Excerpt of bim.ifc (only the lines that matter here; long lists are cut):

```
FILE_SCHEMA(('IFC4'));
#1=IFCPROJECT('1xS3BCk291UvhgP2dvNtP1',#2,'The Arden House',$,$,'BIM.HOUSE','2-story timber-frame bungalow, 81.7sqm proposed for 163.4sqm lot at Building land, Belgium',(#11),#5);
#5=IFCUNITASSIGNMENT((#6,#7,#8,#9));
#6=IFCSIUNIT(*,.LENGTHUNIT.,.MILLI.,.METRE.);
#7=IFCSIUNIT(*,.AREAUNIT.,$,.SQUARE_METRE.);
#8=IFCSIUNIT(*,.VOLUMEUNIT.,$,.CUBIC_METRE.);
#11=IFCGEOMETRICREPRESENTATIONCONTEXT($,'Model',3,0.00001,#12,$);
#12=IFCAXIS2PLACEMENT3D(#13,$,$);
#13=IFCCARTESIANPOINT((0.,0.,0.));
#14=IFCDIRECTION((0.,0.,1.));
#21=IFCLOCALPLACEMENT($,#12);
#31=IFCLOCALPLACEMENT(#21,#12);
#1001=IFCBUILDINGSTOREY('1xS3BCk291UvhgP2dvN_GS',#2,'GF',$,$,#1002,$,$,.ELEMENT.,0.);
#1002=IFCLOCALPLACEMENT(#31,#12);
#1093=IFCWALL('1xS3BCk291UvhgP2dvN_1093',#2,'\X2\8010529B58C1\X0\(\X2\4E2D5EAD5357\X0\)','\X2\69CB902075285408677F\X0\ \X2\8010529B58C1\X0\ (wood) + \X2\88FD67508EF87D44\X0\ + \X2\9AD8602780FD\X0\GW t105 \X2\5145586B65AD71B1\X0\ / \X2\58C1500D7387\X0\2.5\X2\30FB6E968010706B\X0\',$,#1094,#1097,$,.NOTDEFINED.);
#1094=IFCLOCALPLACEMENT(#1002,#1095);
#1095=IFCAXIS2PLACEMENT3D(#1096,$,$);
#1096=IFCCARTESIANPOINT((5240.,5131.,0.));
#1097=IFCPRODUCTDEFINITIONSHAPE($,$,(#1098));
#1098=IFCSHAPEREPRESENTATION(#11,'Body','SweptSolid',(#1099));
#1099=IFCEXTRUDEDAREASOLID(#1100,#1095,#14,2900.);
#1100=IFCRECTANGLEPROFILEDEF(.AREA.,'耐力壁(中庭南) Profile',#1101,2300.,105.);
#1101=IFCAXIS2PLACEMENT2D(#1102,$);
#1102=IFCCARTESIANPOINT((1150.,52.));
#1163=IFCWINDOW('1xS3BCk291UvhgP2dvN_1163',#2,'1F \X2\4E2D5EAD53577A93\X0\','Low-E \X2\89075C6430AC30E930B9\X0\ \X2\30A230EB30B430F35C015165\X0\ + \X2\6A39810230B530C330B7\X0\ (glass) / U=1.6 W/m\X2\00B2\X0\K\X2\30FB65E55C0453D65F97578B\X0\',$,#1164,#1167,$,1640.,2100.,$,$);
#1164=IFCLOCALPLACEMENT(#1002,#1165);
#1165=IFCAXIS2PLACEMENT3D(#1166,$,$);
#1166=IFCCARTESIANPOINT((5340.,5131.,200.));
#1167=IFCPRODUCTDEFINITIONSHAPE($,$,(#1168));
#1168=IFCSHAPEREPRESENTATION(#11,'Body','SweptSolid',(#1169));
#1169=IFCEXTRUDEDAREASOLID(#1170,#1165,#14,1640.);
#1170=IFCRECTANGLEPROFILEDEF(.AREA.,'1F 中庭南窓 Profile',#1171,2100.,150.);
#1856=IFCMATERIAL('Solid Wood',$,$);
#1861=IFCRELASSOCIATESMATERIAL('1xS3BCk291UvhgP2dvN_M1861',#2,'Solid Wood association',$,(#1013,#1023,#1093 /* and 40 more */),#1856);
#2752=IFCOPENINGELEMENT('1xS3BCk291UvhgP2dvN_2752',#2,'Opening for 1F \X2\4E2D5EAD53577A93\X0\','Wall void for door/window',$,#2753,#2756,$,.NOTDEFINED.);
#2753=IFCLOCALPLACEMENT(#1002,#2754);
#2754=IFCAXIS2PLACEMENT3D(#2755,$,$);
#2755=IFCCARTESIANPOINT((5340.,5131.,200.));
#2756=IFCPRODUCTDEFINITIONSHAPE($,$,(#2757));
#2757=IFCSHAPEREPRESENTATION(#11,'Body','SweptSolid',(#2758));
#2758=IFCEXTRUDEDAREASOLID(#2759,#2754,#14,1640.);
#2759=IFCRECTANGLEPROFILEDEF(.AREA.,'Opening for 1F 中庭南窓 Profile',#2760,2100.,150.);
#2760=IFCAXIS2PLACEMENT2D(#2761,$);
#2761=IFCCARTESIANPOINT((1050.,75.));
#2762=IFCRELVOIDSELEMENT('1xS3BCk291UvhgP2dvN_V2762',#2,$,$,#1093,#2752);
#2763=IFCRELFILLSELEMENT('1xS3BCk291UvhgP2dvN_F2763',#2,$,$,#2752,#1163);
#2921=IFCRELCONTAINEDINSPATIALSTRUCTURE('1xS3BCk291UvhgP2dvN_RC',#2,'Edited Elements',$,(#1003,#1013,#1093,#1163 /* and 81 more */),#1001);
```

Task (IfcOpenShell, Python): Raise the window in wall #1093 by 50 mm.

```python
import numpy as np
import ifcopenshell
import ifcopenshell.api.geometry
import ifcopenshell.util.placement
import ifcopenshell.util.unit

model = ifcopenshell.open("bim.ifc")
unit_scale = ifcopenshell.util.unit.calculate_unit_scale(model)

window = model.by_guid("1xS3BCk291UvhgP2dvN_1163")
opening = window.FillsVoids[0].RelatingOpeningElement
dz = 50.0

shift = np.array([0.0, 0.0, dz])
# The window is not placed relative to its opening, so move both.
for product in (opening, window):
    matrix = ifcopenshell.util.placement.get_local_placement(product.ObjectPlacement)
    matrix[:3, 3] += shift
    ifcopenshell.api.geometry.edit_object_placement(model, product=product, matrix=matrix, is_si=False)

print(f"moved by {dz * unit_scale:+.3f} m")

model.write("bim_v2.ifc")
```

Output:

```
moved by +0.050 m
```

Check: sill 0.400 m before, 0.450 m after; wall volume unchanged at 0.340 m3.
